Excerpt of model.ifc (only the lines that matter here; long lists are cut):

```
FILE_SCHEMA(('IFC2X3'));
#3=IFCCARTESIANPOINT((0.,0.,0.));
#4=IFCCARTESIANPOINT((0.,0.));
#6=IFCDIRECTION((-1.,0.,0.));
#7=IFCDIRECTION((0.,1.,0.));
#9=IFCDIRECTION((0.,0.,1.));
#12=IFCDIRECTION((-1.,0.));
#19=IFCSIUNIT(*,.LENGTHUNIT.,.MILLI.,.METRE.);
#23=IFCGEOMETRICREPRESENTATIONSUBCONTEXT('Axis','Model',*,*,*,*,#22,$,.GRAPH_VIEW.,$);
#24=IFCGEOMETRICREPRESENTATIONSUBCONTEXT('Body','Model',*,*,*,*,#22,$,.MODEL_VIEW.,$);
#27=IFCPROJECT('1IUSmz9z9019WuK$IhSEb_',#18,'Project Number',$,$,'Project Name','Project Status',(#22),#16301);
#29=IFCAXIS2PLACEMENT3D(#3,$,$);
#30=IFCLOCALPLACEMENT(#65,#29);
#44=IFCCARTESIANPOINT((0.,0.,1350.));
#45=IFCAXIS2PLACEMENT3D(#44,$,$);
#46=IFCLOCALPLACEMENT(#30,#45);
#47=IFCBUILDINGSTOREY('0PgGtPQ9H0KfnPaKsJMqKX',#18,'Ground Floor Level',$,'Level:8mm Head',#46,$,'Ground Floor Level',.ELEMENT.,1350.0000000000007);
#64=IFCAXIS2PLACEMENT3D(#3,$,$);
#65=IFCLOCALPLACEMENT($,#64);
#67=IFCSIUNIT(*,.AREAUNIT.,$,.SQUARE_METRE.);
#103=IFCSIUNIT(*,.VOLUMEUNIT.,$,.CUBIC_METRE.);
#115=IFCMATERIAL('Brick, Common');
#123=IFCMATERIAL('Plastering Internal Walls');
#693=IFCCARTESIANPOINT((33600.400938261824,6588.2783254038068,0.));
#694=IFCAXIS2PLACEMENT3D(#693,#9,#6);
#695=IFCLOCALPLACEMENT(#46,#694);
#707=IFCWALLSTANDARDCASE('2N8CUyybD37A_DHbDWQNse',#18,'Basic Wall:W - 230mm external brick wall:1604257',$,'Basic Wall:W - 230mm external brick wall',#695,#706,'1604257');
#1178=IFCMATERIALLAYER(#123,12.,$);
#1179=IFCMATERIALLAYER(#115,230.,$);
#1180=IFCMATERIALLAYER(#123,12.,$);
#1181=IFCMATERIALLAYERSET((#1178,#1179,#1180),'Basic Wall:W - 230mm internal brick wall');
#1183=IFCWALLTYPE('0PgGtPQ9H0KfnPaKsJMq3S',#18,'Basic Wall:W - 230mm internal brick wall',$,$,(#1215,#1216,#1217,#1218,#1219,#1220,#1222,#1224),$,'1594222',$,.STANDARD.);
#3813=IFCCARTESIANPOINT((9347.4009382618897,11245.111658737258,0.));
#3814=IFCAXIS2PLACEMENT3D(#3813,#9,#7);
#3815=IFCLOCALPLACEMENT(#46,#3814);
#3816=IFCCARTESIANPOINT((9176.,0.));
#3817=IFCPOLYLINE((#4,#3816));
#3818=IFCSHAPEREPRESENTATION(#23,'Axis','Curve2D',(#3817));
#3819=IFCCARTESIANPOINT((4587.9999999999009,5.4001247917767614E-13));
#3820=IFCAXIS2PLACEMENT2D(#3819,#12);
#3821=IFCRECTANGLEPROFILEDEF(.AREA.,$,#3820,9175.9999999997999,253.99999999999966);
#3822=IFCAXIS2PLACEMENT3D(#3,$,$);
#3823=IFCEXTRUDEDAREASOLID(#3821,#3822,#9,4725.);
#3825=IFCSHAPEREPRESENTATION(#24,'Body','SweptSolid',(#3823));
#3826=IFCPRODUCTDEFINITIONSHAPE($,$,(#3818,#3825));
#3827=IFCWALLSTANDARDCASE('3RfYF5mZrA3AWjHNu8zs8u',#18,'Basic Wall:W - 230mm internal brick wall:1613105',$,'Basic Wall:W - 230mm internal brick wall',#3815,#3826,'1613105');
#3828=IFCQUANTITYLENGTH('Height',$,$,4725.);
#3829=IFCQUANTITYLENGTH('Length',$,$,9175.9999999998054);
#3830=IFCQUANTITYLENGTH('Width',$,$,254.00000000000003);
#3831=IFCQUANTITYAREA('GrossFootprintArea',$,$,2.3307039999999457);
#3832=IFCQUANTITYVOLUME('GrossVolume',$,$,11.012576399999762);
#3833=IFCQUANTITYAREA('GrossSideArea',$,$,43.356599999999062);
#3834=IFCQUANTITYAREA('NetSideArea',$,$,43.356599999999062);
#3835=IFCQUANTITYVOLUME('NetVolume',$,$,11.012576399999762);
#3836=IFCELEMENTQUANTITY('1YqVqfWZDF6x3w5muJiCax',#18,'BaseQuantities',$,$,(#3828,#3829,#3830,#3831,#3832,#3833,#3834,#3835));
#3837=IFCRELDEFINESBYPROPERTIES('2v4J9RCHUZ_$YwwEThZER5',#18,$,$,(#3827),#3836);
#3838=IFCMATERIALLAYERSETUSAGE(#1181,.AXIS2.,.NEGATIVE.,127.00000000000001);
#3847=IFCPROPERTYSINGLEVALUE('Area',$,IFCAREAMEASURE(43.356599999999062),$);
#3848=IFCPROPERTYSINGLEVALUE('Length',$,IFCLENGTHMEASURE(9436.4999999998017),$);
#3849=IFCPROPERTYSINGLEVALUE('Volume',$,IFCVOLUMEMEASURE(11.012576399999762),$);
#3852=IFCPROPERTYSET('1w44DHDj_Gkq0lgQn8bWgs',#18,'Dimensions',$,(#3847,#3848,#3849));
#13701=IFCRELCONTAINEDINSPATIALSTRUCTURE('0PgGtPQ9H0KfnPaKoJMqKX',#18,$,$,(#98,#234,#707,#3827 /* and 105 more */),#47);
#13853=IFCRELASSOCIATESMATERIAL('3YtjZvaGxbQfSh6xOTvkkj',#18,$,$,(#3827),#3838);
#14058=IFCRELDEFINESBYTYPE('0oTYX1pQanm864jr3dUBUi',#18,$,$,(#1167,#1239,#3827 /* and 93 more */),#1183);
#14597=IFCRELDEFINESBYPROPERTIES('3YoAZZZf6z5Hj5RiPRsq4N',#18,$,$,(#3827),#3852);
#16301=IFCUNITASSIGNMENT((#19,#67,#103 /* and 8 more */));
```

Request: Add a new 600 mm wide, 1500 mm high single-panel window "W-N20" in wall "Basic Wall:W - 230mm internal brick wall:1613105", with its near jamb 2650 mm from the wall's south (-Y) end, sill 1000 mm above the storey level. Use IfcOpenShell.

```python
import numpy as np
import ifcopenshell
import ifcopenshell.api.feature
import ifcopenshell.api.geometry
import ifcopenshell.api.pset
import ifcopenshell.api.root
import ifcopenshell.api.spatial
import ifcopenshell.api.type
import ifcopenshell.geom
import ifcopenshell.util.element
import ifcopenshell.util.placement
import ifcopenshell.util.representation
import ifcopenshell.util.shape
import ifcopenshell.util.unit

model = ifcopenshell.open("model.ifc")
unit_scale = ifcopenshell.util.unit.calculate_unit_scale(model)
area_scale = ifcopenshell.util.unit.calculate_unit_scale(model, "AREAUNIT")
volume_scale = ifcopenshell.util.unit.calculate_unit_scale(model, "VOLUMEUNIT")
settings = ifcopenshell.geom.settings()


def volume(element):
    """Net volume in cubic metres, openings subtracted."""
    shape = ifcopenshell.geom.create_shape(settings, element)
    return ifcopenshell.util.shape.get_volume(shape.geometry)


wall = model.by_guid("3RfYF5mZrA3AWjHNu8zs8u")
storey = ifcopenshell.util.element.get_container(wall, ifc_class="IfcBuildingStorey")
context = ifcopenshell.util.representation.get_context(model, "Model", "Body", "MODEL_VIEW")
before = volume(wall)

width, height, from_end, sill = 0.6, 1.5, 2.65, 1  # metres

# The wall runs along its own X axis, and the end named is its -X end.
wall_shape = ifcopenshell.geom.create_shape(settings, wall)
x, y, z = ifcopenshell.util.shape.get_vertices(wall_shape.geometry).T
start = x.min() + from_end
face, thickness = float(y.min()), float(y.max() - y.min())
wall_matrix = ifcopenshell.util.placement.get_local_placement(wall.ObjectPlacement)
level = ifcopenshell.util.placement.get_local_placement(storey.ObjectPlacement)[2, 3]


def in_wall(x, y):
    """Placement at x, y metres in the wall's axes, at sill height."""
    matrix = wall_matrix.copy()
    matrix[:, 3] = wall_matrix @ np.array([x / unit_scale, y / unit_scale, 0.0, 1.0])
    matrix[2, 3] = level + sill / unit_scale
    return matrix


# Opening: a box that overshoots both wall faces by 50 mm.
opening = ifcopenshell.api.root.create_entity(model, ifc_class="IfcOpeningElement")
box = ifcopenshell.api.geometry.add_wall_representation(
    model, context=context, length=width, height=height, thickness=thickness + 0.1
)
ifcopenshell.api.geometry.assign_representation(model, product=opening, representation=box)
ifcopenshell.api.geometry.edit_object_placement(model, product=opening, matrix=in_wall(start, face - 0.05), is_si=False)
ifcopenshell.api.feature.add_feature(model, feature=opening, element=wall)

window = ifcopenshell.api.root.create_entity(model, ifc_class="IfcWindow", name="W-N20")
window.OverallWidth, window.OverallHeight = width / unit_scale, height / unit_scale
body = ifcopenshell.api.geometry.add_window_representation(
    model,
    context=context,
    overall_width=window.OverallWidth,
    overall_height=window.OverallHeight,
    partition_type="SINGLE_PANEL",
)
ifcopenshell.api.geometry.assign_representation(model, product=window, representation=body)
ifcopenshell.api.spatial.assign_container(model, products=[window], relating_structure=storey)
fills = ifcopenshell.api.feature.add_filling(model, opening=opening, element=window)
fills.OwnerHistory = window.OwnerHistory  # required in IFC2X3

# IFC2X3 keeps the operation on the window style.
style = ifcopenshell.api.root.create_entity(model, ifc_class="IfcWindowStyle", name="W-N20")
style.OperationType, style.ConstructionType = "SINGLE_PANEL", "NOTDEFINED"
style.ParameterTakesPrecedence = style.Sizeable = False
ifcopenshell.api.type.assign_type(model, related_objects=[window], relating_type=style)

# Centre the window in the wall's thickness.
ifcopenshell.api.geometry.edit_object_placement(model, product=window, matrix=in_wall(start, face), is_si=False)
window_shape = ifcopenshell.geom.create_shape(settings, window)
depth = ifcopenshell.util.shape.get_vertices(window_shape.geometry)[:, 1]
offset = face + thickness / 2 - (depth.min() + depth.max()) / 2
ifcopenshell.api.geometry.edit_object_placement(model, product=window, matrix=in_wall(start, offset), is_si=False)

after = volume(wall)

# Update the wall's stored quantities.
qto = model.by_id(ifcopenshell.util.element.get_pset(wall, "BaseQuantities", should_inherit=False)["id"])
ifcopenshell.api.pset.edit_qto(model, qto=qto, properties={
    "NetSideArea": after / thickness / area_scale,
    "NetVolume": after / volume_scale,
})
pset = model.by_id(ifcopenshell.util.element.get_pset(wall, "Dimensions", should_inherit=False)["id"])
ifcopenshell.api.pset.edit_pset(model, pset=pset, properties={
    "Area": model.create_entity("IfcAreaMeasure", after / thickness / area_scale),
    "Volume": model.create_entity("IfcVolumeMeasure", after / volume_scale),
})

print(f"wall volume {before:.3f} -> {after:.3f} m3")

model.write("model-out.ifc")
```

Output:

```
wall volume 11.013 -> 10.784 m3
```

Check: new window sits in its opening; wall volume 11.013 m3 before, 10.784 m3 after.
